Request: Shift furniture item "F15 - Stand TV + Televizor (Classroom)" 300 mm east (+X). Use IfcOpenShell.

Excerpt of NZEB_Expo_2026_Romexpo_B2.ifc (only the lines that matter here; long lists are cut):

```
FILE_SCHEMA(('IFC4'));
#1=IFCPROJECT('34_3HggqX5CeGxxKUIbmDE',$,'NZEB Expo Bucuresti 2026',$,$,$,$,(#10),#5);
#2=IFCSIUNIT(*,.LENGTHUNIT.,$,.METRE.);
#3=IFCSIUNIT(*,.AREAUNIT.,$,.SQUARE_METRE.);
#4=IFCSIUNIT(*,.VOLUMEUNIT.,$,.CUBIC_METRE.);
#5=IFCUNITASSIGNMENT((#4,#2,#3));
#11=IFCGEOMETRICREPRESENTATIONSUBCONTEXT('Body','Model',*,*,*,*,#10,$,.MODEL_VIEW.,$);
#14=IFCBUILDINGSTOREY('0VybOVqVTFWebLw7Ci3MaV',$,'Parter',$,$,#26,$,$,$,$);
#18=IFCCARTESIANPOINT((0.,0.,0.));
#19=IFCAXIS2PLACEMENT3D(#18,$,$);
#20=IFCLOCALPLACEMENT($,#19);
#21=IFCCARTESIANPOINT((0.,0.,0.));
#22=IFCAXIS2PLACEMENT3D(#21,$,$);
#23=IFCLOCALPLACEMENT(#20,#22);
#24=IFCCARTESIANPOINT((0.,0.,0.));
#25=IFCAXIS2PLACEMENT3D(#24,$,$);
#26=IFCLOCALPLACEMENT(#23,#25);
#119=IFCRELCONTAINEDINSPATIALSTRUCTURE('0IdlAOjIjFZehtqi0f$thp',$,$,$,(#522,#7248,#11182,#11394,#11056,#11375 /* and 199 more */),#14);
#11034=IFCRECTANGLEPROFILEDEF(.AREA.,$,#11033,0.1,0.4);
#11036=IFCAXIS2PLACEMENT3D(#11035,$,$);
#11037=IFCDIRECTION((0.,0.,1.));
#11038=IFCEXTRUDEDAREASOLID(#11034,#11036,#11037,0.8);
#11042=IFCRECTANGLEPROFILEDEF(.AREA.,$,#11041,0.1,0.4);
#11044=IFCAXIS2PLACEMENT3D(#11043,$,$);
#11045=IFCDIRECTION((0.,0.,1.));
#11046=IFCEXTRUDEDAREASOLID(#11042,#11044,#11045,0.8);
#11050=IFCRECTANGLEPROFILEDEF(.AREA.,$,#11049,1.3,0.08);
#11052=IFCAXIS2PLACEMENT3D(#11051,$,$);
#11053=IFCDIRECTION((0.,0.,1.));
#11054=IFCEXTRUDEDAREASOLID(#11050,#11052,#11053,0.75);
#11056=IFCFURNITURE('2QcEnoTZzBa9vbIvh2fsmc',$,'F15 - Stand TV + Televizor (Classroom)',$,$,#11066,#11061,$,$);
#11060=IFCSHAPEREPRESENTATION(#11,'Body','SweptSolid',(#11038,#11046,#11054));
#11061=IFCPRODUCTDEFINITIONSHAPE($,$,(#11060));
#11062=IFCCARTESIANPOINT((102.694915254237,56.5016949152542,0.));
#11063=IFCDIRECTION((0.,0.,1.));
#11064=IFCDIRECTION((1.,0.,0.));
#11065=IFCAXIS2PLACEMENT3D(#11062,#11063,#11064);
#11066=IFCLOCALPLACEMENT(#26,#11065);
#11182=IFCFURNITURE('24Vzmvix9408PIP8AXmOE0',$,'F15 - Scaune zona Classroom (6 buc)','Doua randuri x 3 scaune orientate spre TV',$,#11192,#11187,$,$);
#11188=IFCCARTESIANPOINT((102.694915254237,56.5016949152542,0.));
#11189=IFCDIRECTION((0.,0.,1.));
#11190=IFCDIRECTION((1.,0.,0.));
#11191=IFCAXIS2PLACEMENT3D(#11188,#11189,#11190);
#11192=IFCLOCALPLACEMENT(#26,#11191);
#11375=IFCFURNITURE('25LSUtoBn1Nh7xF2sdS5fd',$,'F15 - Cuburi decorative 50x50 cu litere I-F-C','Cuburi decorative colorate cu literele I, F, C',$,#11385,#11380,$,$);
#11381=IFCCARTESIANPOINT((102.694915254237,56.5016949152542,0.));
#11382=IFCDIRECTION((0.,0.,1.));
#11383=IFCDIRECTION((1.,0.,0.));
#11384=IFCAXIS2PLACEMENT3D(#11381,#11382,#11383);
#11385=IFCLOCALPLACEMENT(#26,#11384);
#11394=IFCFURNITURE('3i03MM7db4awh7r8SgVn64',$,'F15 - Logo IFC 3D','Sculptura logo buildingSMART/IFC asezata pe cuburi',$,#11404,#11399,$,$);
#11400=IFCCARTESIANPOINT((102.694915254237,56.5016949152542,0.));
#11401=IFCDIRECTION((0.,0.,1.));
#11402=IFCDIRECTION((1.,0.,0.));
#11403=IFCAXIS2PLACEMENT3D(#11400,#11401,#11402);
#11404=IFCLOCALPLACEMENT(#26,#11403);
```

```python
import ifcopenshell
import ifcopenshell.api.geometry
import ifcopenshell.util.placement
import ifcopenshell.util.unit

model = ifcopenshell.open("NZEB_Expo_2026_Romexpo_B2.ifc")
unit_scale = ifcopenshell.util.unit.calculate_unit_scale(model)

item = model.by_id(11056)
matrix = ifcopenshell.util.placement.get_local_placement(item.ObjectPlacement)
matrix[0, 3] += 0.3 / unit_scale
ifcopenshell.api.geometry.edit_object_placement(model, product=item, matrix=matrix, is_si=False)

print(ifcopenshell.util.placement.get_local_placement(item.ObjectPlacement).round(3) + 0.0)

model.write("NZEB_Expo_2026_Romexpo_B2_v2.ifc")
```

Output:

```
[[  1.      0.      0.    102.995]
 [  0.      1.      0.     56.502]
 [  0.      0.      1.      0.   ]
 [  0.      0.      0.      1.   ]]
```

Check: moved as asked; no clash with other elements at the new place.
